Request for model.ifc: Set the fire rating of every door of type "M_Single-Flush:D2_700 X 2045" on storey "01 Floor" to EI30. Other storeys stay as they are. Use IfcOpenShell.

First a look at what the model holds.

```python
import ifcopenshell
import ifcopenshell.util.element

model = ifcopenshell.open("model.ifc")
print(model.schema)
storey = next(s for s in model.by_type("IfcBuildingStorey") if s.Name == "01 Floor")
doors = [e for e in ifcopenshell.util.element.get_decomposition(storey) if e.is_a("IfcDoor")]
seen = {}
for e in doors:
    element_type = ifcopenshell.util.element.get_type(e)
    key = (element_type.Name if element_type != e and element_type else None, ifcopenshell.util.element.get_pset(e, "Pset_DoorCommon", "FireRating"))
    seen[key] = seen.get(key, 0) + 1
for (name, value), count in sorted(seen.items(), key=str):
    print(count, "x", name, "|", value)
```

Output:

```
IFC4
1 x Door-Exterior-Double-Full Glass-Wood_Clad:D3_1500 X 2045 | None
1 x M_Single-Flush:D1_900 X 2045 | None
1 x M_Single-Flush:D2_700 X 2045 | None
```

```python
import ifcopenshell
import ifcopenshell.api.pset
import ifcopenshell.util.element

model = ifcopenshell.open("model.ifc")

storey = next(s for s in model.by_type("IfcBuildingStorey") if s.Name == "01 Floor")
doors = [e for e in ifcopenshell.util.element.get_decomposition(storey) if e.is_a("IfcDoor")]

count = 0
for e in doors:
    element_type = ifcopenshell.util.element.get_type(e)
    if element_type in (None, e) or element_type.Name != "M_Single-Flush:D2_700 X 2045":
        continue
    # add_pset returns the element's existing set when there is one.
    pset = ifcopenshell.api.pset.add_pset(model, product=e, name="Pset_DoorCommon")
    ifcopenshell.api.pset.edit_pset(model, pset=pset, properties={"FireRating": "EI30"})
    count += 1

print(count, "doors updated")

model.write("model-out.ifc")
```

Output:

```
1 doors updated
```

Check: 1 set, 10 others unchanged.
